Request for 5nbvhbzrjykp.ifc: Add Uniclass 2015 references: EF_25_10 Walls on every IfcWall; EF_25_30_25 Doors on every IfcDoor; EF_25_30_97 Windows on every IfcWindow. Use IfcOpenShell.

First a look at what the model holds.

```python
import ifcopenshell

model = ifcopenshell.open("5nbvhbzrjykp.ifc")
print(model.schema)
print("classifications:", [c.Name for c in model.by_type("IfcClassification")])
for ifc_class in ("IfcDoor", "IfcRoof", "IfcStair", "IfcWall", "IfcWindow"):
    print(ifc_class, len(model.by_type(ifc_class)))
```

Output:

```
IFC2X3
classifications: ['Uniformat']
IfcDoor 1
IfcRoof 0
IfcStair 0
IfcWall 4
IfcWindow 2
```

```python
import ifcopenshell
import ifcopenshell.api.classification

model = ifcopenshell.open("5nbvhbzrjykp.ifc")

# IFC2X3 requires Source and Edition and has no link from the project to the system.
system = model.create_entity("IfcClassification", Source="NBS", Edition="2015", Name="Uniclass 2015")

codes = {
    "IfcWall": ("EF_25_10", "Walls"),
    "IfcDoor": ("EF_25_30_25", "Doors"),
    "IfcWindow": ("EF_25_30_97", "Windows"),
}
for ifc_class, (code, name) in codes.items():
    products = model.by_type(ifc_class)
    ifcopenshell.api.classification.add_reference(
        model, products=products, classification=system, identification=code, name=name
    )
    print(code, len(products))

model.write("5nbvhbzrjykp-out.ifc")
```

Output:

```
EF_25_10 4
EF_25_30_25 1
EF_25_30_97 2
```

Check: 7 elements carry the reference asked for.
